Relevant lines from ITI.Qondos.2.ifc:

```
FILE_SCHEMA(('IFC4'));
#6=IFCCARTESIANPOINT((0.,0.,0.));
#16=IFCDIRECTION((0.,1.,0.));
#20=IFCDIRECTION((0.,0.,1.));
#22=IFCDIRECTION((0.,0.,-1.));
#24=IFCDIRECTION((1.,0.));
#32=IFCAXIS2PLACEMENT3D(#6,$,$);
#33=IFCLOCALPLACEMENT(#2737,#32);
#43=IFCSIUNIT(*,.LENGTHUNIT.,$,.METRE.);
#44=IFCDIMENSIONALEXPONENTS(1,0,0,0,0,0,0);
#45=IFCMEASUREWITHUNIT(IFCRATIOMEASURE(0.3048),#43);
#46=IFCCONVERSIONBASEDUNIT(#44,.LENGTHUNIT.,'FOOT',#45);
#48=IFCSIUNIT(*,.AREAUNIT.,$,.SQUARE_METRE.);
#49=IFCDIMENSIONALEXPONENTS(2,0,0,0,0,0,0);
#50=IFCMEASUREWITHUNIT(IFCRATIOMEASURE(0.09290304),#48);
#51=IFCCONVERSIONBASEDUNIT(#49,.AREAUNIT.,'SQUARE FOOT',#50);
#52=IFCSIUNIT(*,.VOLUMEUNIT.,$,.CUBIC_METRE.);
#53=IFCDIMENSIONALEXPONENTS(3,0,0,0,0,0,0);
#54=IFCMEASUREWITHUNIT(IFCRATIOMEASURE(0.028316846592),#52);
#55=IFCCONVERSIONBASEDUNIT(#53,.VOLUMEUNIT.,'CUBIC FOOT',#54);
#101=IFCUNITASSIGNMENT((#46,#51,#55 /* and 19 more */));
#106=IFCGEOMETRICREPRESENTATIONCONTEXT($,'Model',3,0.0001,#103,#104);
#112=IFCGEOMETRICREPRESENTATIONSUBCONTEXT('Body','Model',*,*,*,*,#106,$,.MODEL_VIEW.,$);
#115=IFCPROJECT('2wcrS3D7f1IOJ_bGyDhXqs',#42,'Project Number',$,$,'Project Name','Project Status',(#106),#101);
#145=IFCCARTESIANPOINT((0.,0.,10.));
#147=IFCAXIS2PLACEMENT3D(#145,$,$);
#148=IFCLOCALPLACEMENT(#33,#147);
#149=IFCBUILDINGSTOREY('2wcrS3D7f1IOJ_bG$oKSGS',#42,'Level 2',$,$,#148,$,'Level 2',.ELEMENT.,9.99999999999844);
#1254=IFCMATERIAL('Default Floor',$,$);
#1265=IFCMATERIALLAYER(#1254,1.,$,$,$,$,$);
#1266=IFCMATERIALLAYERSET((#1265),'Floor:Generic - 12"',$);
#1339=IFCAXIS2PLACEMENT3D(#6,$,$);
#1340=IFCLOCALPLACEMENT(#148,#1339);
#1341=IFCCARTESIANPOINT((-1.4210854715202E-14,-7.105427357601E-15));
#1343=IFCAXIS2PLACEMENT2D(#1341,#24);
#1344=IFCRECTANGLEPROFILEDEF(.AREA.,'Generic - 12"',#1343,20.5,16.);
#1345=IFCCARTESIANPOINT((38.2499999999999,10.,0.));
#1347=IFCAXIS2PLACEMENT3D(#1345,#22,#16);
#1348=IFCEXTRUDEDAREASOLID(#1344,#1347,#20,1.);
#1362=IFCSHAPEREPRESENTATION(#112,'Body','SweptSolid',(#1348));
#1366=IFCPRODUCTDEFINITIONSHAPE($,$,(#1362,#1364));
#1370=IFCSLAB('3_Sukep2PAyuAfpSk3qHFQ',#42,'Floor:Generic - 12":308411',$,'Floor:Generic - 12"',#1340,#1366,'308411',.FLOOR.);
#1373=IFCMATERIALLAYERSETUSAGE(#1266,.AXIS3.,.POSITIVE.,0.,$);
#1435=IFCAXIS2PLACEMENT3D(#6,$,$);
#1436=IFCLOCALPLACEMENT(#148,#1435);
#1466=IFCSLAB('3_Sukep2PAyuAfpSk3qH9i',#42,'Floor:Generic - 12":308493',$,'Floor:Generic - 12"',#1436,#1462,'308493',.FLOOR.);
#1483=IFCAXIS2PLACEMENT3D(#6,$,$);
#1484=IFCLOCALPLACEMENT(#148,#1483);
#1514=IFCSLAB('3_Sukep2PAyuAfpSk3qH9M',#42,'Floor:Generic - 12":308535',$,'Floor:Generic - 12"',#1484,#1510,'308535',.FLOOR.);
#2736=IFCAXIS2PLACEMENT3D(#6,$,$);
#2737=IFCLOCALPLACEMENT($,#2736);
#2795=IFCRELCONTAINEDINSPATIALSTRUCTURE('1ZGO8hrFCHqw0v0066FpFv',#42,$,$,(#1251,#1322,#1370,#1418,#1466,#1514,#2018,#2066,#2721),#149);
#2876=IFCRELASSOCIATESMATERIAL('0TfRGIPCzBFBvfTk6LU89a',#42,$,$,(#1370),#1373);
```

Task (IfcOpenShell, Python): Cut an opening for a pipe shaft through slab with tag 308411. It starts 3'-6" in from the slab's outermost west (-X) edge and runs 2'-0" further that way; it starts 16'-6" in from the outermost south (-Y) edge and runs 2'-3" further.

```python
import numpy as np
import ifcopenshell
import ifcopenshell.api.feature
import ifcopenshell.api.geometry
import ifcopenshell.api.root
import ifcopenshell.geom
import ifcopenshell.util.placement
import ifcopenshell.util.representation
import ifcopenshell.util.shape
import ifcopenshell.util.unit

model = ifcopenshell.open("ITI.Qondos.2.ifc")
unit_scale = ifcopenshell.util.unit.calculate_unit_scale(model)
settings = ifcopenshell.geom.settings()


def volume(element):
    """Net volume in cubic metres, openings subtracted."""
    shape = ifcopenshell.geom.create_shape(settings, element)
    return ifcopenshell.util.shape.get_volume(shape.geometry)


slab = model.by_guid("3_Sukep2PAyuAfpSk3qHFQ")
before = volume(slab)

# Extent in the slab's own axes, in metres. The edges named are its -X and -Y sides.
slab_shape = ifcopenshell.geom.create_shape(settings, slab)
vertices = ifcopenshell.util.shape.get_vertices(slab_shape.geometry)
x_min, y_min, bottom = vertices.min(axis=0)
top = vertices[:, 2].max()

opening = ifcopenshell.api.root.create_entity(model, ifc_class="IfcOpeningElement", name="Pipe shaft opening", predefined_type="OPENING")
context = ifcopenshell.util.representation.get_context(model, "Model", "Body", "MODEL_VIEW")
width, depth = 0.6096, 0.6858
outline = [(0.0, 0.0), (width, 0.0), (width, depth), (0.0, depth), (0.0, 0.0)]
# Overshoot both faces by 50 mm so the cut is clean.
shape = ifcopenshell.api.geometry.add_slab_representation(
    model, context=context, depth=top - bottom + 0.1, polyline=outline
)
ifcopenshell.api.geometry.assign_representation(model, product=opening, representation=shape)

matrix = ifcopenshell.util.placement.get_local_placement(slab.ObjectPlacement)
matrix[:, 3] = matrix @ np.append(np.array([x_min + 1.0668, y_min + 5.0292, bottom - 0.05]) / unit_scale, 1.0)
ifcopenshell.api.geometry.edit_object_placement(model, product=opening, matrix=matrix, is_si=False)
ifcopenshell.api.feature.add_feature(model, feature=opening, element=slab)

after = volume(slab)

print(f"slab volume {before:.3f} -> {after:.3f} m3")

model.write("ITI.Qondos.2_updated.ifc")
```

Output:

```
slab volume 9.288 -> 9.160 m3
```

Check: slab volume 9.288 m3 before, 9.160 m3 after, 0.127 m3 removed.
